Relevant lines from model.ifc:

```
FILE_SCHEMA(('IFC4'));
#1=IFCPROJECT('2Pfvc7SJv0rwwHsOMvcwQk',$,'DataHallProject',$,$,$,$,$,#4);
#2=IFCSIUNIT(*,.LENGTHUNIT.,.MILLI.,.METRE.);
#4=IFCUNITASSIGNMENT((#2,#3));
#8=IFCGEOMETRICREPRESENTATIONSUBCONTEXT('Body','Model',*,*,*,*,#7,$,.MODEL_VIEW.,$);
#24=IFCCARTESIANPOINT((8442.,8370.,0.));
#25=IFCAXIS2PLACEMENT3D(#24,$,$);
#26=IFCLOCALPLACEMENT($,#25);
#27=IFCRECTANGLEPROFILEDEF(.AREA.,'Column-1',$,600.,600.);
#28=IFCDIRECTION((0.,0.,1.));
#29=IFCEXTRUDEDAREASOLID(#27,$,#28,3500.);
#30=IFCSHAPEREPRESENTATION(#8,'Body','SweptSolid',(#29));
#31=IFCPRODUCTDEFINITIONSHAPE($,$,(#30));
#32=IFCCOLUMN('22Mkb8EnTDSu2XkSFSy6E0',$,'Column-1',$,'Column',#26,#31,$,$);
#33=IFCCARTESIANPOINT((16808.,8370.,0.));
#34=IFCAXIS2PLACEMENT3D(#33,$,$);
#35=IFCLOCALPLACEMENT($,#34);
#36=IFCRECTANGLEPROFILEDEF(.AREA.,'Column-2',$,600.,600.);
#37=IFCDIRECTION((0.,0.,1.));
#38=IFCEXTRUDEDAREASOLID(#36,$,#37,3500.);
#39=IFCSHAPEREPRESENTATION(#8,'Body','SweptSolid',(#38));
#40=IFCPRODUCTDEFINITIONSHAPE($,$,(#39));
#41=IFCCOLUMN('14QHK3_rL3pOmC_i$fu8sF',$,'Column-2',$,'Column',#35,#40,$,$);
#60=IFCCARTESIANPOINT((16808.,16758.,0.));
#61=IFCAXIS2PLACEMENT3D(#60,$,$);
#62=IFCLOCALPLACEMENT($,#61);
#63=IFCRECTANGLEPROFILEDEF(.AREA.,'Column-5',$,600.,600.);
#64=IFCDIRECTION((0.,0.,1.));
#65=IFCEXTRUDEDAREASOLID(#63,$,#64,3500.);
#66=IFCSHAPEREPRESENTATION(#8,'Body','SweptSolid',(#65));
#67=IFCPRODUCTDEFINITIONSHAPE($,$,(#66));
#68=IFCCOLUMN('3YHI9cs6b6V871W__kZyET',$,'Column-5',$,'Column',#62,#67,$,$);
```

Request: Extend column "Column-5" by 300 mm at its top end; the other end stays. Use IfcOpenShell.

```python
import ifcopenshell
import ifcopenshell.util.representation

model = ifcopenshell.open("model.ifc")

member = model.by_guid("3YHI9cs6b6V871W__kZyET")
change = 300.0

# The extrusion runs towards the end named, so only its depth changes.
body = ifcopenshell.util.representation.get_representation(member, "Model", "Body")
solid = body.Items[0]
old_length = solid.Depth
solid.Depth += change

print(f"length {old_length:g} -> {solid.Depth:g}")

model.write("model-out.ifc")
```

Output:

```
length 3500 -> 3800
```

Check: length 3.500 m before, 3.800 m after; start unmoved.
